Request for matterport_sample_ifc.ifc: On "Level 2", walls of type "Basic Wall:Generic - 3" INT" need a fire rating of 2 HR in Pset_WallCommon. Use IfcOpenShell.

First a look at what the model holds.

```python
import ifcopenshell
import ifcopenshell.util.element

model = ifcopenshell.open("matterport_sample_ifc.ifc")
print(model.schema)
storey = next(s for s in model.by_type("IfcBuildingStorey") if s.Name == "Level 2")
walls = [e for e in ifcopenshell.util.element.get_decomposition(storey) if e.is_a("IfcWall")]
seen = {}
for e in walls:
    element_type = ifcopenshell.util.element.get_type(e)
    key = (element_type.Name if element_type != e and element_type else None, ifcopenshell.util.element.get_pset(e, "Pset_WallCommon", "FireRating"))
    seen[key] = seen.get(key, 0) + 1
for (name, value), count in sorted(seen.items(), key=str):
    print(count, "x", name, "|", value)
```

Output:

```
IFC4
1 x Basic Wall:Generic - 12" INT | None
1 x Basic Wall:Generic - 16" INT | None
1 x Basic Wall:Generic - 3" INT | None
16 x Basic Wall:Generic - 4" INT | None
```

```python
import ifcopenshell
import ifcopenshell.api.pset
import ifcopenshell.util.element

model = ifcopenshell.open("matterport_sample_ifc.ifc")

storey = next(s for s in model.by_type("IfcBuildingStorey") if s.Name == "Level 2")
walls = [e for e in ifcopenshell.util.element.get_decomposition(storey) if e.is_a("IfcWall")]

count = 0
for e in walls:
    element_type = ifcopenshell.util.element.get_type(e)
    if element_type in (None, e) or element_type.Name != 'Basic Wall:Generic - 3" INT':
        continue
    # add_pset returns the element's existing set when there is one.
    pset = ifcopenshell.api.pset.add_pset(model, product=e, name="Pset_WallCommon")
    ifcopenshell.api.pset.edit_pset(model, pset=pset, properties={"FireRating": "2 HR"})
    count += 1

print(count, "walls updated")

model.write("matterport_sample_ifc_rev.ifc")
```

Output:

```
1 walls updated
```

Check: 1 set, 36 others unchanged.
